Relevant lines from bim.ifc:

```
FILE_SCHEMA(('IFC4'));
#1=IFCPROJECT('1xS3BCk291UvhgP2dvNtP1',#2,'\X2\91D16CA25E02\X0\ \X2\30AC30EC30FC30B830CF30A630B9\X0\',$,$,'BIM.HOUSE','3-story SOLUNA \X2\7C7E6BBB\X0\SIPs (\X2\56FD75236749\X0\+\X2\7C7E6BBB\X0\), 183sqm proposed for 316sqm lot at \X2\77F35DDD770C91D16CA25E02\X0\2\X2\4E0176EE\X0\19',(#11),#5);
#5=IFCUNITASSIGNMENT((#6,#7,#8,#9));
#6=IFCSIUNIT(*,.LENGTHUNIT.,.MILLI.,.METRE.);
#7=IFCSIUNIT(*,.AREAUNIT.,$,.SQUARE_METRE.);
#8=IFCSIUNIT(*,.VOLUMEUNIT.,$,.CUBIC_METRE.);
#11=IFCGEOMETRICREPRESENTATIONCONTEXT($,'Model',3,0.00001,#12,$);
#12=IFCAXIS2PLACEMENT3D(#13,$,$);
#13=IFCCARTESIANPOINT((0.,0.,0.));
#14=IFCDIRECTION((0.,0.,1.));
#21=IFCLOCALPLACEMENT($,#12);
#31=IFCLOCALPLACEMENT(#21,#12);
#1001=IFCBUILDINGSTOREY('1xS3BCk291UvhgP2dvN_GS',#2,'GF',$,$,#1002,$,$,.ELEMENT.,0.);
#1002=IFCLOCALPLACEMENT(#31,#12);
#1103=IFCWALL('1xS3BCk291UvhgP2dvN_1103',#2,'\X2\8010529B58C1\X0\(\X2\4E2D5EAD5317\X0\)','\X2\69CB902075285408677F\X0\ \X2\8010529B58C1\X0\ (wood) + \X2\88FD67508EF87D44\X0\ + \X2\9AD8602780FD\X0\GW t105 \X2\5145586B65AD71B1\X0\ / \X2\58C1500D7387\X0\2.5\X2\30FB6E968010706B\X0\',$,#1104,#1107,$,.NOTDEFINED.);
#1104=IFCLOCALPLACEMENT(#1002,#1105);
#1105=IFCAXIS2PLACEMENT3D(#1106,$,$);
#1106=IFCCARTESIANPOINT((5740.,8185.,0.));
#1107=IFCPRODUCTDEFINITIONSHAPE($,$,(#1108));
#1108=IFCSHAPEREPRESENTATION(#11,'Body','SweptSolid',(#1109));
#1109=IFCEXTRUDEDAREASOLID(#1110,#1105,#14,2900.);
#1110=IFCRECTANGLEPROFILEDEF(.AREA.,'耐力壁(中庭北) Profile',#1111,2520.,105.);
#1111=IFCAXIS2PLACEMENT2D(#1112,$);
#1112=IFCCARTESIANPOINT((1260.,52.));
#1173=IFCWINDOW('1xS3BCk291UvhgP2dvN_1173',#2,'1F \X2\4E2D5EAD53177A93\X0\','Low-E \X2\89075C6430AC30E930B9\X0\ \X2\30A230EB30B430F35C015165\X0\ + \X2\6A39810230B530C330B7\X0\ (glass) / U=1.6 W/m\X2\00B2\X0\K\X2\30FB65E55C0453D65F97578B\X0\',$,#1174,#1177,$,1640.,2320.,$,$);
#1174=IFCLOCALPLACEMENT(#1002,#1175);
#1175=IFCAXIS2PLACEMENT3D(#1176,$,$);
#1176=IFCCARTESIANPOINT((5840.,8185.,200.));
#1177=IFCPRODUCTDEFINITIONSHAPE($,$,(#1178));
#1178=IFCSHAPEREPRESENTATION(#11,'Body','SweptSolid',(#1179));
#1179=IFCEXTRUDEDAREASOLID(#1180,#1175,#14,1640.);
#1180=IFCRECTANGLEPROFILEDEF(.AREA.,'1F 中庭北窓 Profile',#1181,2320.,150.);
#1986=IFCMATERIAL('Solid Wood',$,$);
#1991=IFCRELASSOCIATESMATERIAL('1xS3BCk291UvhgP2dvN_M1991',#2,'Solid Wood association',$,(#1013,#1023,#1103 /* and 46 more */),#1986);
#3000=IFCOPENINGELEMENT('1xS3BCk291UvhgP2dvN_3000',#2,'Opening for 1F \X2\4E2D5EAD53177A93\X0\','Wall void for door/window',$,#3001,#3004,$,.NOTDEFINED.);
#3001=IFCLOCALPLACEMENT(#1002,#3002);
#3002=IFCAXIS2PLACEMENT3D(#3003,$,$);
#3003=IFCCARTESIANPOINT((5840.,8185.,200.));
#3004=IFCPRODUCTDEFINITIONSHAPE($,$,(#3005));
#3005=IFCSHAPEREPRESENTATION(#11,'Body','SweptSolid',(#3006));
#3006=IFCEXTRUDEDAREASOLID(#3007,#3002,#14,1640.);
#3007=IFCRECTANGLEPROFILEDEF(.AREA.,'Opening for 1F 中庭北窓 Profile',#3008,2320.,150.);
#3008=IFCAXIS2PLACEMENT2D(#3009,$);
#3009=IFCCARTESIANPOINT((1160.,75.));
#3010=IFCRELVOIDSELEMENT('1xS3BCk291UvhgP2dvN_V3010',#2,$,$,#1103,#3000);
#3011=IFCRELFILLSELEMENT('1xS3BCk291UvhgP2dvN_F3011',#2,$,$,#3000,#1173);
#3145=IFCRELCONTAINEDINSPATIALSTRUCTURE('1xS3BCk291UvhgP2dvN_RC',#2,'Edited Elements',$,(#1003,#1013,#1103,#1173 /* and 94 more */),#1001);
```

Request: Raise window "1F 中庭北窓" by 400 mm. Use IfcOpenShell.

```python
import numpy as np
import ifcopenshell
import ifcopenshell.api.geometry
import ifcopenshell.util.placement
import ifcopenshell.util.unit

model = ifcopenshell.open("bim.ifc")
unit_scale = ifcopenshell.util.unit.calculate_unit_scale(model)

window = model.by_id(1173)
opening = window.FillsVoids[0].RelatingOpeningElement
dz = 0.4 / unit_scale

shift = np.array([0.0, 0.0, dz])
# The window is not placed relative to its opening, so move both.
for product in (opening, window):
    matrix = ifcopenshell.util.placement.get_local_placement(product.ObjectPlacement)
    matrix[:3, 3] += shift
    ifcopenshell.api.geometry.edit_object_placement(model, product=product, matrix=matrix, is_si=False)

print(f"moved by {dz * unit_scale:+.3f} m")

model.write("bim_rev.ifc")
```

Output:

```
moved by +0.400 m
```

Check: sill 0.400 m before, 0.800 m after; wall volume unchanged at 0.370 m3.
